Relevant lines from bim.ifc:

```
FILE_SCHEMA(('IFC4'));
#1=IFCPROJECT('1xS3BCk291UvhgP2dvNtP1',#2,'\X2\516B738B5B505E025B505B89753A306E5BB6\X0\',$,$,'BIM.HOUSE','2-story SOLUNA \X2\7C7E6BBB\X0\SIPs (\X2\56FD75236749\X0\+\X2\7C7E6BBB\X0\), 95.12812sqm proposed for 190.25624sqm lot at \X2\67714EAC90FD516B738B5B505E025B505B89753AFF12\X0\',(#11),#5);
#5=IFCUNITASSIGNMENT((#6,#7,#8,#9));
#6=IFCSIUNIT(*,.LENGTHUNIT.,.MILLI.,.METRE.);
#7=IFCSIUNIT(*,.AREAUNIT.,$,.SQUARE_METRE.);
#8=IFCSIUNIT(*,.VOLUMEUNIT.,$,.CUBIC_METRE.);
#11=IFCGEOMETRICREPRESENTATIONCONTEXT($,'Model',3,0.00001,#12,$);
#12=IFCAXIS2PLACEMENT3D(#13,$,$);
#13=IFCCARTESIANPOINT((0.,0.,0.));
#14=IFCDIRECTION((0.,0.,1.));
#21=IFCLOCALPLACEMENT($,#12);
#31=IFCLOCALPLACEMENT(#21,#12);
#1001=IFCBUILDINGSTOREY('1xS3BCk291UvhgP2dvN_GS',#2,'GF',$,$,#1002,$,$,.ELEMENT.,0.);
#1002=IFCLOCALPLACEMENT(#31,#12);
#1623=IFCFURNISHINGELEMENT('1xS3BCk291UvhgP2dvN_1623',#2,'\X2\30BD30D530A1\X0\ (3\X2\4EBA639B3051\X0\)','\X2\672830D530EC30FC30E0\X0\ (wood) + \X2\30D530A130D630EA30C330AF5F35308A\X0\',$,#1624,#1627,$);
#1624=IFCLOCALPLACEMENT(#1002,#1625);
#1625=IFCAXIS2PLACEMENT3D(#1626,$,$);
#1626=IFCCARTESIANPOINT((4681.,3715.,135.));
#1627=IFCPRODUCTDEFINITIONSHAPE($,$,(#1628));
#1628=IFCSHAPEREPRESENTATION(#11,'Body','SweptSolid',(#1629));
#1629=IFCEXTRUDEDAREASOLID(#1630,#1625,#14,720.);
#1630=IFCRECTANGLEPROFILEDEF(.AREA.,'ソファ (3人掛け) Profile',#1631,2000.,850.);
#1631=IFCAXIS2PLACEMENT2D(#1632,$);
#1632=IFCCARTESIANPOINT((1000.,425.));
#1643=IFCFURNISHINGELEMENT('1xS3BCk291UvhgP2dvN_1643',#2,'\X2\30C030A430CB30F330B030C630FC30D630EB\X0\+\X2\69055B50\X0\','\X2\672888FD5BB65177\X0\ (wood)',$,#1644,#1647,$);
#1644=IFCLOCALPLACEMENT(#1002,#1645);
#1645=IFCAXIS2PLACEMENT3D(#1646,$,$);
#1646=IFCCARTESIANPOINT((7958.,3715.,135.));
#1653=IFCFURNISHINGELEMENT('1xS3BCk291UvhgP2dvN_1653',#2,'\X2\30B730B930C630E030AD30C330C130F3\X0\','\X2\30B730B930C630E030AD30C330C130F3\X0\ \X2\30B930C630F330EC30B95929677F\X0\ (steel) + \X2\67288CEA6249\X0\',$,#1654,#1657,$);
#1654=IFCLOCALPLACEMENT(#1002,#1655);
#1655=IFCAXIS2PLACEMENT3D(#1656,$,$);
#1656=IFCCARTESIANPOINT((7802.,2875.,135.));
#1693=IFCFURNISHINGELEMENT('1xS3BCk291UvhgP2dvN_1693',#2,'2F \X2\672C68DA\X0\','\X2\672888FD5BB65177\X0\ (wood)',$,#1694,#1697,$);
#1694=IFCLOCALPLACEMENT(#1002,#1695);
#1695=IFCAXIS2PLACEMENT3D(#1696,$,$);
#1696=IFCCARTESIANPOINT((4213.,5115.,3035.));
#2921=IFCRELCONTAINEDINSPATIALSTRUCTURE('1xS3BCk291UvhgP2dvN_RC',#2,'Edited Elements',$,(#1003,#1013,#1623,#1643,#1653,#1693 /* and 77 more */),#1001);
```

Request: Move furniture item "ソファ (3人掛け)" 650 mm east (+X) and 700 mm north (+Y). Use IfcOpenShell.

```python
import ifcopenshell
import ifcopenshell.api.geometry
import ifcopenshell.util.placement

model = ifcopenshell.open("bim.ifc")

item = model.by_id(1623)
matrix = ifcopenshell.util.placement.get_local_placement(item.ObjectPlacement)
matrix[0, 3] += 650.0
matrix[1, 3] += 700.0
ifcopenshell.api.geometry.edit_object_placement(model, product=item, matrix=matrix, is_si=False)

print(ifcopenshell.util.placement.get_local_placement(item.ObjectPlacement).round(3) + 0.0)

model.write("bim_edited.ifc")
```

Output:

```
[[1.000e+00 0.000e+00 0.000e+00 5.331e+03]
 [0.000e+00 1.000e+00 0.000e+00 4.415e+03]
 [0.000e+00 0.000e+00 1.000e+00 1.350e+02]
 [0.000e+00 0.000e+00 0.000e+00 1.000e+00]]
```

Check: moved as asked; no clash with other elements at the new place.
